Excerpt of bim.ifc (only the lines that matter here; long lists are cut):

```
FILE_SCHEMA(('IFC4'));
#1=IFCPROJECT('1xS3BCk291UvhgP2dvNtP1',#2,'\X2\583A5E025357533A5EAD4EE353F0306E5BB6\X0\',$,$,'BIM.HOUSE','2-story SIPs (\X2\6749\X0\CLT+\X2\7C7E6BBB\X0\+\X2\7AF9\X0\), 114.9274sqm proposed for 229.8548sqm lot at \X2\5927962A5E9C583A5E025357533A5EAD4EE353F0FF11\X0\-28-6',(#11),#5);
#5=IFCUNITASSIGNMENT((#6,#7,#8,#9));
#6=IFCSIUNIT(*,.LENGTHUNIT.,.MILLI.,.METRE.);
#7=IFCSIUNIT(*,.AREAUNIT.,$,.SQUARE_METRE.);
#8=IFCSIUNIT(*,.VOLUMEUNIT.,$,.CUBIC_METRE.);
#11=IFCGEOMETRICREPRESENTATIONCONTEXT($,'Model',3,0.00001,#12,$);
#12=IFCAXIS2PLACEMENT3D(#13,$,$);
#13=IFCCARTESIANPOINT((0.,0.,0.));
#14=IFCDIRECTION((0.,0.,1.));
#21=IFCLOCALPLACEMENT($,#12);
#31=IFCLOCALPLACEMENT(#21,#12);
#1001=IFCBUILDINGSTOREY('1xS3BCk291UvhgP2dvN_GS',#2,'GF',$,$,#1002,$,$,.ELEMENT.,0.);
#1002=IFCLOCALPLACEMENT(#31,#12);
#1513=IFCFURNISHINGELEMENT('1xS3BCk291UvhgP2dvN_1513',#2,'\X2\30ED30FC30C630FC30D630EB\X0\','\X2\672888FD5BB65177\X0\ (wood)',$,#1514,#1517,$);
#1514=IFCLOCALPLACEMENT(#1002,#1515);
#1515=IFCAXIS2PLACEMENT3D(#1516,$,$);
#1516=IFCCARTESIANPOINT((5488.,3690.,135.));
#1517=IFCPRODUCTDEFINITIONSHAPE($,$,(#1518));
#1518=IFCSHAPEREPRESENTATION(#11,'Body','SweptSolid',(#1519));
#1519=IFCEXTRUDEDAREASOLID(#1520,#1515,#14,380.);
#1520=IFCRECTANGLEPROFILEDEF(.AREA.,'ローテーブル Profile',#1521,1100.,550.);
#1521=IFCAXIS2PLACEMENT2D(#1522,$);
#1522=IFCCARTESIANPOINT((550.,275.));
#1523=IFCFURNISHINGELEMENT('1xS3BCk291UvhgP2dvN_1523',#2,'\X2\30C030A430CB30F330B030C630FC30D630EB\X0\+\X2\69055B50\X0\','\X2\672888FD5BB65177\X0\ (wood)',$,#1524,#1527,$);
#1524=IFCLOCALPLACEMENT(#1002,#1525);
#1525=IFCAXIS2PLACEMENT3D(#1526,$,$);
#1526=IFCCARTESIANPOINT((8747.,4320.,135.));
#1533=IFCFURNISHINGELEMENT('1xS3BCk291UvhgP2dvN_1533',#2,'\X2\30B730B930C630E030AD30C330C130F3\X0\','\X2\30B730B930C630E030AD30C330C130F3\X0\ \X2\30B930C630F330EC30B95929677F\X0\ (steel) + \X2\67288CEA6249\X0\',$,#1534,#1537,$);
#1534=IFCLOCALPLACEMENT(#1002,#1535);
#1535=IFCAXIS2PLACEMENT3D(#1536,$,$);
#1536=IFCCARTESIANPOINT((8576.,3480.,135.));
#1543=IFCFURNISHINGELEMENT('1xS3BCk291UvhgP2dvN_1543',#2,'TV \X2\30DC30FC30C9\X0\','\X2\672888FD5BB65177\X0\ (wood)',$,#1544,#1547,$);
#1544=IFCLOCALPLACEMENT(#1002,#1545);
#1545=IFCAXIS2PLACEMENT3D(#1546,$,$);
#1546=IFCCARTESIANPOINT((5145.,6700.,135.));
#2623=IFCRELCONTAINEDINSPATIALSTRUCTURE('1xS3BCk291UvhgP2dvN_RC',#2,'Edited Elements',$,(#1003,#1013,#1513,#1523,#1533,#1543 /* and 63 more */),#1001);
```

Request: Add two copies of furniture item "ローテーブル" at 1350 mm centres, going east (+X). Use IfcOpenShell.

```python
import numpy as np
import ifcopenshell
import ifcopenshell.api.geometry
import ifcopenshell.api.root
import ifcopenshell.util.element
import ifcopenshell.util.placement
import ifcopenshell.util.unit

model = ifcopenshell.open("bim.ifc")
unit_scale = ifcopenshell.util.unit.calculate_unit_scale(model)


def reuse_history(source, copy):
    """copy_class also copies each property set's owner history, people and application; keep the originals."""
    for rel in copy.IsDefinedBy:
        if rel.is_a("IfcRelDefinesByProperties") and (history := rel.RelatingPropertyDefinition.OwnerHistory):
            rel.RelatingPropertyDefinition.OwnerHistory = source.OwnerHistory
            ifcopenshell.util.element.remove_deep2(model, history)


source = model.by_id(1513)
base = ifcopenshell.util.placement.get_local_placement(source.ObjectPlacement)
step = np.array([1.0, 0.0, 0.0]) * 1.35 / unit_scale

for i in range(1, 3):
    copy = ifcopenshell.api.root.copy_class(model, product=source)
    copy.Representation = ifcopenshell.util.element.copy_deep(
        model, source.Representation, exclude=["IfcGeometricRepresentationContext", "IfcRepresentationMap"]
    )
    reuse_history(source, copy)
    matrix = base.copy()
    matrix[:3, 3] += i * step
    print("added at", matrix[:3, 3].round(3) + 0.0)
    ifcopenshell.api.geometry.edit_object_placement(model, product=copy, matrix=matrix, is_si=False)

model.write("bim_updated.ifc")
```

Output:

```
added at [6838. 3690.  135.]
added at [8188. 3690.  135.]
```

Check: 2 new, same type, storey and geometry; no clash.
